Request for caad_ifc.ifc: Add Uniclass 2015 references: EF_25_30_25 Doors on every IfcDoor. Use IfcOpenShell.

First a look at what the model holds.

```python
import ifcopenshell

model = ifcopenshell.open("caad_ifc.ifc")
print(model.schema)
print("classifications:", [c.Name for c in model.by_type("IfcClassification")])
for ifc_class in ("IfcDoor", "IfcRoof", "IfcStair", "IfcWall", "IfcWindow"):
    print(ifc_class, len(model.by_type(ifc_class)))
```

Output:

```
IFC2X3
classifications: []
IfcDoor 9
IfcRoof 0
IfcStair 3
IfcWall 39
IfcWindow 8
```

```python
import ifcopenshell
import ifcopenshell.api.classification

model = ifcopenshell.open("caad_ifc.ifc")

# IFC2X3 requires Source and Edition and has no link from the project to the system.
system = model.create_entity("IfcClassification", Source="NBS", Edition="2015", Name="Uniclass 2015")

codes = {
    "IfcDoor": ("EF_25_30_25", "Doors"),
}
for ifc_class, (code, name) in codes.items():
    products = model.by_type(ifc_class)
    ifcopenshell.api.classification.add_reference(
        model, products=products, classification=system, identification=code, name=name
    )
    print(code, len(products))

model.write("caad_ifc-out.ifc")
```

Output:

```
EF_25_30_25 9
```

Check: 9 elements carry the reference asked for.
